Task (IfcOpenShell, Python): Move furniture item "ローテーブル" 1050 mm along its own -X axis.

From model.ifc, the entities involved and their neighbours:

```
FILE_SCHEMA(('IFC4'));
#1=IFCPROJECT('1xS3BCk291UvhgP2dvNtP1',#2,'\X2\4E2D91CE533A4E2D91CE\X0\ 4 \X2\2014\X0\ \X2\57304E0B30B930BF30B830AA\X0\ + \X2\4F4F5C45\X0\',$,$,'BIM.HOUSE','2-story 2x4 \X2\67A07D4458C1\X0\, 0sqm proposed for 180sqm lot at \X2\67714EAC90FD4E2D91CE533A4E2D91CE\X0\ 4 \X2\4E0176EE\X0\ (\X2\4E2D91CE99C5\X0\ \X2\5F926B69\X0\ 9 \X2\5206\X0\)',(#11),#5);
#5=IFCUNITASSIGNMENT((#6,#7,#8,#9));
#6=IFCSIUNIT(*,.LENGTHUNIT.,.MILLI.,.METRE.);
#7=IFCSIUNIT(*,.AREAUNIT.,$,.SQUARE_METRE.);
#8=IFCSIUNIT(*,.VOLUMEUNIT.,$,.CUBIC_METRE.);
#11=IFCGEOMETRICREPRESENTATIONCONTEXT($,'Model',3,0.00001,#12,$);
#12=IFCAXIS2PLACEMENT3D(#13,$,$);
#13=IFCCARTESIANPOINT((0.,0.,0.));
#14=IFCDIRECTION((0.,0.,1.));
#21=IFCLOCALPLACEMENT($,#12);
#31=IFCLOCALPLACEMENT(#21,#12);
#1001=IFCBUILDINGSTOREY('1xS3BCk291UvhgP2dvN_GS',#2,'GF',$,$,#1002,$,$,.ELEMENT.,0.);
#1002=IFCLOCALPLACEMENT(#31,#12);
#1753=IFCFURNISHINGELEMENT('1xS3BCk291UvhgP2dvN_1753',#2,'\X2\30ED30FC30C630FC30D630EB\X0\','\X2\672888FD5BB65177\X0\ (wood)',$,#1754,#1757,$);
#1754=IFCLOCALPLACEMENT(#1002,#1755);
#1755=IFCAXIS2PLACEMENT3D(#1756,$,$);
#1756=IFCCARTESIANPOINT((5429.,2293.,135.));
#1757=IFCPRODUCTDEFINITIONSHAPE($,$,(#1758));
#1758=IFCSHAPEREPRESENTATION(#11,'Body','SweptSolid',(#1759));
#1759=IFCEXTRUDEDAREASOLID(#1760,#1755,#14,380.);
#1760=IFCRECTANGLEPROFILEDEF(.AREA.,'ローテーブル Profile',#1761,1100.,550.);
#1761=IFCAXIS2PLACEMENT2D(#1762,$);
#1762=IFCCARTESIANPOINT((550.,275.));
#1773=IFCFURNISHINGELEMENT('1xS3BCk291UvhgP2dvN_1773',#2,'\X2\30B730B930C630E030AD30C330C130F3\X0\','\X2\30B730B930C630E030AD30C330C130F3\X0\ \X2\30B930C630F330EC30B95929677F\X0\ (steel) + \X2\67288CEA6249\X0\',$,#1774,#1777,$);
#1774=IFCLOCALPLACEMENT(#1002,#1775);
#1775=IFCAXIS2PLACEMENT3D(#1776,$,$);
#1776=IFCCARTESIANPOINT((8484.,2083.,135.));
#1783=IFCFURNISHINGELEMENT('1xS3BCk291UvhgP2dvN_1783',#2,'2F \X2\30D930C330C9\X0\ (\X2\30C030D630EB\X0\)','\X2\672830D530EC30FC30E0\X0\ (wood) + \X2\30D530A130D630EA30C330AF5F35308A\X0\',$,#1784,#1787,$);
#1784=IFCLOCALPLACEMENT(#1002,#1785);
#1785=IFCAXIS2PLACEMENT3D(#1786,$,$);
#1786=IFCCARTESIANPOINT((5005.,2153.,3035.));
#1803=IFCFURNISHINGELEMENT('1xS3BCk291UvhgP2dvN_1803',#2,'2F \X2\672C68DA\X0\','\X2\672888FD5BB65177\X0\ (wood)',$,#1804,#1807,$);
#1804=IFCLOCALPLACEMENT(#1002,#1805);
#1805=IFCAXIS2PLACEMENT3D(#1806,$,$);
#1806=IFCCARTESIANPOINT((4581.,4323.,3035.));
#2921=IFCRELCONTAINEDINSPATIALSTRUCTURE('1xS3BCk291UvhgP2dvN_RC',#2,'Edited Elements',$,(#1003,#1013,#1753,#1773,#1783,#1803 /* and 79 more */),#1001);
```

```python
import ifcopenshell
import ifcopenshell.api.geometry
import ifcopenshell.util.placement
import ifcopenshell.util.unit

model = ifcopenshell.open("model.ifc")
unit_scale = ifcopenshell.util.unit.calculate_unit_scale(model)

item = model.by_guid("1xS3BCk291UvhgP2dvN_1753")
matrix = ifcopenshell.util.placement.get_local_placement(item.ObjectPlacement)
matrix[:3, 3] -= matrix[:3, 0] * 1.05 / unit_scale
ifcopenshell.api.geometry.edit_object_placement(model, product=item, matrix=matrix, is_si=False)

print(ifcopenshell.util.placement.get_local_placement(item.ObjectPlacement).round(3) + 0.0)

model.write("model_updated.ifc")
```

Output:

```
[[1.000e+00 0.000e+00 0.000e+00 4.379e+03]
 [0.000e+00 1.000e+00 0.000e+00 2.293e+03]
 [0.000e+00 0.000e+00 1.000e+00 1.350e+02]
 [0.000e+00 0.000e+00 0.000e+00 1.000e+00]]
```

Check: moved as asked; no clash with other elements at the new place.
